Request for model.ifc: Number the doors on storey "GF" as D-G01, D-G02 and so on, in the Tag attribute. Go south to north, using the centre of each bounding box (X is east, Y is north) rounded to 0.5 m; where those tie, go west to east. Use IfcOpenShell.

First a look at what the model holds.

```python
import ifcopenshell
import ifcopenshell.util.element
import ifcopenshell.util.placement

model = ifcopenshell.open("model.ifc")
print(model.schema)
storey = next(s for s in model.by_type("IfcBuildingStorey") if s.Name == "GF")
doors = [e for e in ifcopenshell.util.element.get_decomposition(storey) if e.is_a("IfcDoor")]
for e in sorted(doors, key=lambda e: e.id()):
    origin = ifcopenshell.util.placement.get_local_placement(e.ObjectPlacement)[:3, 3]
    print(e.id(), e.Tag, e.Name, origin.round(2) + 0.0, sep=" | ")
```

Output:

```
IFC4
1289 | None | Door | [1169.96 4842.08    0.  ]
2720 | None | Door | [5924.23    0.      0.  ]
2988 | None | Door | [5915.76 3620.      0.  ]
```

```python
import ifcopenshell
import ifcopenshell.geom
import ifcopenshell.util.element
import ifcopenshell.util.shape

model = ifcopenshell.open("model.ifc")
settings = ifcopenshell.geom.settings()
settings.set("use-world-coords", True)


def centre(element):
    shape = ifcopenshell.geom.create_shape(settings, element)
    return ifcopenshell.util.shape.get_bbox_centroid(shape.geometry)


storey = next(s for s in model.by_type("IfcBuildingStorey") if s.Name == "GF")
doors = [e for e in ifcopenshell.util.element.get_decomposition(storey) if e.is_a("IfcDoor")]

# Insertion points can sit at a corner or the storey origin, so sort by the geometry (in metres).
centres = {e: centre(e) for e in doors}
doors.sort(key=lambda e: (round(centres[e][1] / 0.5), centres[e][0]))

for i, e in enumerate(doors, start=1):
    number = f"D-G{i:02d}"
    e.Tag = number
    print(e.id(), number)

model.write("model_updated.ifc")
```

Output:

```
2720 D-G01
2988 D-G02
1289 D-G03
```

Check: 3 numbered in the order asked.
